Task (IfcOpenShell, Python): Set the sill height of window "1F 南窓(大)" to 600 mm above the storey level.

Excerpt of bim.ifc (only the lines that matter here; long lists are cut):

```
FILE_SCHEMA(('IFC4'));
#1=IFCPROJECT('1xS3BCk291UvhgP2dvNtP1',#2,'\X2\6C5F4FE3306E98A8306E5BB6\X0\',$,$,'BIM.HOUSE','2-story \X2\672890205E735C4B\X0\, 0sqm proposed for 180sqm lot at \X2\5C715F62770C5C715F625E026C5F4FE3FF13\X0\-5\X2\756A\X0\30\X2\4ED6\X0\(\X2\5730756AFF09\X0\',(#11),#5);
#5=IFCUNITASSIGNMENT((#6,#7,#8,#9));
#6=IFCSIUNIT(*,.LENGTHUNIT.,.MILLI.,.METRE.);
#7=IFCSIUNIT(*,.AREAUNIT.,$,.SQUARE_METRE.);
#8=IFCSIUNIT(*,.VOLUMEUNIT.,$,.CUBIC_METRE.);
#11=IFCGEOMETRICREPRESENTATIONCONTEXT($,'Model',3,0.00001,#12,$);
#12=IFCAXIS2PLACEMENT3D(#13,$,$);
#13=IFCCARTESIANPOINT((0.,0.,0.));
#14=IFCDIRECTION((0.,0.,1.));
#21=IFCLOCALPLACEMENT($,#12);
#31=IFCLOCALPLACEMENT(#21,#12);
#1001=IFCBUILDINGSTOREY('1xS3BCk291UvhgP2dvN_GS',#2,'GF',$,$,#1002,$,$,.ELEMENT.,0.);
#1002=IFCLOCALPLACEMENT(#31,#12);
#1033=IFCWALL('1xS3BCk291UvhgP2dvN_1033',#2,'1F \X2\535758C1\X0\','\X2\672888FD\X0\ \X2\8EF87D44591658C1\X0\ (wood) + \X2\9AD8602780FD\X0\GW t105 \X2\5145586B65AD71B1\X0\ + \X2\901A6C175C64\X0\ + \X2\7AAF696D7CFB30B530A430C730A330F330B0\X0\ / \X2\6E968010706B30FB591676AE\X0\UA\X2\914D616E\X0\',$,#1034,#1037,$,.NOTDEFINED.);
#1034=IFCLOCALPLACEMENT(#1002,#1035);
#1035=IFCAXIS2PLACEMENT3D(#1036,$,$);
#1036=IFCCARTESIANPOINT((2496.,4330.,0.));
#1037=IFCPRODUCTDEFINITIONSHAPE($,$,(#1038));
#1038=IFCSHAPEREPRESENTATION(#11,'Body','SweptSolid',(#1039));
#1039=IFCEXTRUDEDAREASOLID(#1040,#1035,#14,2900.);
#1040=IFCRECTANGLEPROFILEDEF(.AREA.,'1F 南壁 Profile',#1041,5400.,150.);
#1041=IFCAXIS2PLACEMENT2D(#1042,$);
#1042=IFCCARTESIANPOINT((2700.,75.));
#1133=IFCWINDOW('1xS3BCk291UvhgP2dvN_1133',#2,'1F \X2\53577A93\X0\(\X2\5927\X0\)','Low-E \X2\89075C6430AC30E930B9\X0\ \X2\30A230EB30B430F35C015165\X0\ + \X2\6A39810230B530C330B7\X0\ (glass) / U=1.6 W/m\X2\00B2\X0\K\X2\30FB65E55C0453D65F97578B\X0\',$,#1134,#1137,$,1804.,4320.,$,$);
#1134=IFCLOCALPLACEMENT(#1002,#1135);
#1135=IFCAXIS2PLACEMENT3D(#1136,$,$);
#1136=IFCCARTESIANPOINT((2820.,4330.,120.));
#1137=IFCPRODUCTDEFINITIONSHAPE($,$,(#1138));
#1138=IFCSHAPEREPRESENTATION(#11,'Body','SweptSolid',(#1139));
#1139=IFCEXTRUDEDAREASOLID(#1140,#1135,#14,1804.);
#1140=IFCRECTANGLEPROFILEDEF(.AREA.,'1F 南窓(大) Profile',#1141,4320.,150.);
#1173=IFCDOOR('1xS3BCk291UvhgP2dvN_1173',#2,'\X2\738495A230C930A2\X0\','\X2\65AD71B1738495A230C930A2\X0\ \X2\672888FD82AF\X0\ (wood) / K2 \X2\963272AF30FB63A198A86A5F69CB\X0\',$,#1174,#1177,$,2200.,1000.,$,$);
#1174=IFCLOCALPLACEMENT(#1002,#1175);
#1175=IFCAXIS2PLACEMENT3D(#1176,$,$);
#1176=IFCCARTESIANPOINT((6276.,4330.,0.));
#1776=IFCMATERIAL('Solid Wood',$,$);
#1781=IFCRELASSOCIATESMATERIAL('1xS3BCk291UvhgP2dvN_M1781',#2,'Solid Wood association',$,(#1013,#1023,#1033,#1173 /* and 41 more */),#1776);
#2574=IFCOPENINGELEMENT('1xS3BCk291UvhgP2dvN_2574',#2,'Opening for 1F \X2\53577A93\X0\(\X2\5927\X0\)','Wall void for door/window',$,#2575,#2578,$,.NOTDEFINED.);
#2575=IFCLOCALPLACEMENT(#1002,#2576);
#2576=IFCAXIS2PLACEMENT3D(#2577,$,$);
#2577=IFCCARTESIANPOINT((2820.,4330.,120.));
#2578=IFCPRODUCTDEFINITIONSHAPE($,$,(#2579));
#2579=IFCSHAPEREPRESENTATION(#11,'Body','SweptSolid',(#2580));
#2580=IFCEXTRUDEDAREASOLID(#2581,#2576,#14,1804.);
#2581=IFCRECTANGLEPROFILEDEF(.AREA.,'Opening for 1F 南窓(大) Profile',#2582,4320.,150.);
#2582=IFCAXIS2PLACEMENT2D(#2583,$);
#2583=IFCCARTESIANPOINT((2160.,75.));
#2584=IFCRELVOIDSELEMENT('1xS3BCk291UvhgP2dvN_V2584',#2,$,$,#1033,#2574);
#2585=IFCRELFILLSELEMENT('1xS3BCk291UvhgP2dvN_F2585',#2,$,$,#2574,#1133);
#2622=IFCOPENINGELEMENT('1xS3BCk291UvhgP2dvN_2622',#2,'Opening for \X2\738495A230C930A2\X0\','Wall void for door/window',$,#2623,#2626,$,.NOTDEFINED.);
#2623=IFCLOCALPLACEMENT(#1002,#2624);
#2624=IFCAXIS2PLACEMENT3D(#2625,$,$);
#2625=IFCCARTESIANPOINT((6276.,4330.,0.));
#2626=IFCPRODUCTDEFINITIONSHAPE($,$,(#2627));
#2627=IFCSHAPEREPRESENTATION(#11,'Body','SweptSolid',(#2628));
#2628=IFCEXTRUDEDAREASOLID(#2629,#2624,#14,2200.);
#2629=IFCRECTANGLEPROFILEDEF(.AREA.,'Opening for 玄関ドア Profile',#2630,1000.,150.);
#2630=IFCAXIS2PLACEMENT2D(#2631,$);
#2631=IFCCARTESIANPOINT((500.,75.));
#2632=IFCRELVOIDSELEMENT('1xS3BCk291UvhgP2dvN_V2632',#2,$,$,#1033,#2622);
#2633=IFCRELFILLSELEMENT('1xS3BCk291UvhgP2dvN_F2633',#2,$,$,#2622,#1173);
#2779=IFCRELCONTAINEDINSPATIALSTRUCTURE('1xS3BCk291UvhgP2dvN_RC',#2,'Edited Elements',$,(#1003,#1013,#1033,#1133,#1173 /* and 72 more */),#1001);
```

```python
import numpy as np
import ifcopenshell
import ifcopenshell.api.geometry
import ifcopenshell.geom
import ifcopenshell.util.element
import ifcopenshell.util.placement
import ifcopenshell.util.shape
import ifcopenshell.util.unit

model = ifcopenshell.open("bim.ifc")
unit_scale = ifcopenshell.util.unit.calculate_unit_scale(model)

window = model.by_guid("1xS3BCk291UvhgP2dvN_1133")
opening = window.FillsVoids[0].RelatingOpeningElement
storey = ifcopenshell.util.element.get_container(window, ifc_class="IfcBuildingStorey")
level = ifcopenshell.util.placement.get_local_placement(storey.ObjectPlacement)[2, 3]

# The opening's origin need not be at the sill, so measure its lowest point.
shape = ifcopenshell.geom.create_shape(ifcopenshell.geom.settings(), opening)
bottom = ifcopenshell.util.shape.get_shape_bottom_elevation(shape, shape.geometry) / unit_scale
dz = level + 0.6 / unit_scale - bottom

shift = np.array([0.0, 0.0, dz])
# The window is not placed relative to its opening, so move both.
for product in (opening, window):
    matrix = ifcopenshell.util.placement.get_local_placement(product.ObjectPlacement)
    matrix[:3, 3] += shift
    ifcopenshell.api.geometry.edit_object_placement(model, product=product, matrix=matrix, is_si=False)

print(f"moved by {dz * unit_scale:+.3f} m")

model.write("bim_v2.ifc")
```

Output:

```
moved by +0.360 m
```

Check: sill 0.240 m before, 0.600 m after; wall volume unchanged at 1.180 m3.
